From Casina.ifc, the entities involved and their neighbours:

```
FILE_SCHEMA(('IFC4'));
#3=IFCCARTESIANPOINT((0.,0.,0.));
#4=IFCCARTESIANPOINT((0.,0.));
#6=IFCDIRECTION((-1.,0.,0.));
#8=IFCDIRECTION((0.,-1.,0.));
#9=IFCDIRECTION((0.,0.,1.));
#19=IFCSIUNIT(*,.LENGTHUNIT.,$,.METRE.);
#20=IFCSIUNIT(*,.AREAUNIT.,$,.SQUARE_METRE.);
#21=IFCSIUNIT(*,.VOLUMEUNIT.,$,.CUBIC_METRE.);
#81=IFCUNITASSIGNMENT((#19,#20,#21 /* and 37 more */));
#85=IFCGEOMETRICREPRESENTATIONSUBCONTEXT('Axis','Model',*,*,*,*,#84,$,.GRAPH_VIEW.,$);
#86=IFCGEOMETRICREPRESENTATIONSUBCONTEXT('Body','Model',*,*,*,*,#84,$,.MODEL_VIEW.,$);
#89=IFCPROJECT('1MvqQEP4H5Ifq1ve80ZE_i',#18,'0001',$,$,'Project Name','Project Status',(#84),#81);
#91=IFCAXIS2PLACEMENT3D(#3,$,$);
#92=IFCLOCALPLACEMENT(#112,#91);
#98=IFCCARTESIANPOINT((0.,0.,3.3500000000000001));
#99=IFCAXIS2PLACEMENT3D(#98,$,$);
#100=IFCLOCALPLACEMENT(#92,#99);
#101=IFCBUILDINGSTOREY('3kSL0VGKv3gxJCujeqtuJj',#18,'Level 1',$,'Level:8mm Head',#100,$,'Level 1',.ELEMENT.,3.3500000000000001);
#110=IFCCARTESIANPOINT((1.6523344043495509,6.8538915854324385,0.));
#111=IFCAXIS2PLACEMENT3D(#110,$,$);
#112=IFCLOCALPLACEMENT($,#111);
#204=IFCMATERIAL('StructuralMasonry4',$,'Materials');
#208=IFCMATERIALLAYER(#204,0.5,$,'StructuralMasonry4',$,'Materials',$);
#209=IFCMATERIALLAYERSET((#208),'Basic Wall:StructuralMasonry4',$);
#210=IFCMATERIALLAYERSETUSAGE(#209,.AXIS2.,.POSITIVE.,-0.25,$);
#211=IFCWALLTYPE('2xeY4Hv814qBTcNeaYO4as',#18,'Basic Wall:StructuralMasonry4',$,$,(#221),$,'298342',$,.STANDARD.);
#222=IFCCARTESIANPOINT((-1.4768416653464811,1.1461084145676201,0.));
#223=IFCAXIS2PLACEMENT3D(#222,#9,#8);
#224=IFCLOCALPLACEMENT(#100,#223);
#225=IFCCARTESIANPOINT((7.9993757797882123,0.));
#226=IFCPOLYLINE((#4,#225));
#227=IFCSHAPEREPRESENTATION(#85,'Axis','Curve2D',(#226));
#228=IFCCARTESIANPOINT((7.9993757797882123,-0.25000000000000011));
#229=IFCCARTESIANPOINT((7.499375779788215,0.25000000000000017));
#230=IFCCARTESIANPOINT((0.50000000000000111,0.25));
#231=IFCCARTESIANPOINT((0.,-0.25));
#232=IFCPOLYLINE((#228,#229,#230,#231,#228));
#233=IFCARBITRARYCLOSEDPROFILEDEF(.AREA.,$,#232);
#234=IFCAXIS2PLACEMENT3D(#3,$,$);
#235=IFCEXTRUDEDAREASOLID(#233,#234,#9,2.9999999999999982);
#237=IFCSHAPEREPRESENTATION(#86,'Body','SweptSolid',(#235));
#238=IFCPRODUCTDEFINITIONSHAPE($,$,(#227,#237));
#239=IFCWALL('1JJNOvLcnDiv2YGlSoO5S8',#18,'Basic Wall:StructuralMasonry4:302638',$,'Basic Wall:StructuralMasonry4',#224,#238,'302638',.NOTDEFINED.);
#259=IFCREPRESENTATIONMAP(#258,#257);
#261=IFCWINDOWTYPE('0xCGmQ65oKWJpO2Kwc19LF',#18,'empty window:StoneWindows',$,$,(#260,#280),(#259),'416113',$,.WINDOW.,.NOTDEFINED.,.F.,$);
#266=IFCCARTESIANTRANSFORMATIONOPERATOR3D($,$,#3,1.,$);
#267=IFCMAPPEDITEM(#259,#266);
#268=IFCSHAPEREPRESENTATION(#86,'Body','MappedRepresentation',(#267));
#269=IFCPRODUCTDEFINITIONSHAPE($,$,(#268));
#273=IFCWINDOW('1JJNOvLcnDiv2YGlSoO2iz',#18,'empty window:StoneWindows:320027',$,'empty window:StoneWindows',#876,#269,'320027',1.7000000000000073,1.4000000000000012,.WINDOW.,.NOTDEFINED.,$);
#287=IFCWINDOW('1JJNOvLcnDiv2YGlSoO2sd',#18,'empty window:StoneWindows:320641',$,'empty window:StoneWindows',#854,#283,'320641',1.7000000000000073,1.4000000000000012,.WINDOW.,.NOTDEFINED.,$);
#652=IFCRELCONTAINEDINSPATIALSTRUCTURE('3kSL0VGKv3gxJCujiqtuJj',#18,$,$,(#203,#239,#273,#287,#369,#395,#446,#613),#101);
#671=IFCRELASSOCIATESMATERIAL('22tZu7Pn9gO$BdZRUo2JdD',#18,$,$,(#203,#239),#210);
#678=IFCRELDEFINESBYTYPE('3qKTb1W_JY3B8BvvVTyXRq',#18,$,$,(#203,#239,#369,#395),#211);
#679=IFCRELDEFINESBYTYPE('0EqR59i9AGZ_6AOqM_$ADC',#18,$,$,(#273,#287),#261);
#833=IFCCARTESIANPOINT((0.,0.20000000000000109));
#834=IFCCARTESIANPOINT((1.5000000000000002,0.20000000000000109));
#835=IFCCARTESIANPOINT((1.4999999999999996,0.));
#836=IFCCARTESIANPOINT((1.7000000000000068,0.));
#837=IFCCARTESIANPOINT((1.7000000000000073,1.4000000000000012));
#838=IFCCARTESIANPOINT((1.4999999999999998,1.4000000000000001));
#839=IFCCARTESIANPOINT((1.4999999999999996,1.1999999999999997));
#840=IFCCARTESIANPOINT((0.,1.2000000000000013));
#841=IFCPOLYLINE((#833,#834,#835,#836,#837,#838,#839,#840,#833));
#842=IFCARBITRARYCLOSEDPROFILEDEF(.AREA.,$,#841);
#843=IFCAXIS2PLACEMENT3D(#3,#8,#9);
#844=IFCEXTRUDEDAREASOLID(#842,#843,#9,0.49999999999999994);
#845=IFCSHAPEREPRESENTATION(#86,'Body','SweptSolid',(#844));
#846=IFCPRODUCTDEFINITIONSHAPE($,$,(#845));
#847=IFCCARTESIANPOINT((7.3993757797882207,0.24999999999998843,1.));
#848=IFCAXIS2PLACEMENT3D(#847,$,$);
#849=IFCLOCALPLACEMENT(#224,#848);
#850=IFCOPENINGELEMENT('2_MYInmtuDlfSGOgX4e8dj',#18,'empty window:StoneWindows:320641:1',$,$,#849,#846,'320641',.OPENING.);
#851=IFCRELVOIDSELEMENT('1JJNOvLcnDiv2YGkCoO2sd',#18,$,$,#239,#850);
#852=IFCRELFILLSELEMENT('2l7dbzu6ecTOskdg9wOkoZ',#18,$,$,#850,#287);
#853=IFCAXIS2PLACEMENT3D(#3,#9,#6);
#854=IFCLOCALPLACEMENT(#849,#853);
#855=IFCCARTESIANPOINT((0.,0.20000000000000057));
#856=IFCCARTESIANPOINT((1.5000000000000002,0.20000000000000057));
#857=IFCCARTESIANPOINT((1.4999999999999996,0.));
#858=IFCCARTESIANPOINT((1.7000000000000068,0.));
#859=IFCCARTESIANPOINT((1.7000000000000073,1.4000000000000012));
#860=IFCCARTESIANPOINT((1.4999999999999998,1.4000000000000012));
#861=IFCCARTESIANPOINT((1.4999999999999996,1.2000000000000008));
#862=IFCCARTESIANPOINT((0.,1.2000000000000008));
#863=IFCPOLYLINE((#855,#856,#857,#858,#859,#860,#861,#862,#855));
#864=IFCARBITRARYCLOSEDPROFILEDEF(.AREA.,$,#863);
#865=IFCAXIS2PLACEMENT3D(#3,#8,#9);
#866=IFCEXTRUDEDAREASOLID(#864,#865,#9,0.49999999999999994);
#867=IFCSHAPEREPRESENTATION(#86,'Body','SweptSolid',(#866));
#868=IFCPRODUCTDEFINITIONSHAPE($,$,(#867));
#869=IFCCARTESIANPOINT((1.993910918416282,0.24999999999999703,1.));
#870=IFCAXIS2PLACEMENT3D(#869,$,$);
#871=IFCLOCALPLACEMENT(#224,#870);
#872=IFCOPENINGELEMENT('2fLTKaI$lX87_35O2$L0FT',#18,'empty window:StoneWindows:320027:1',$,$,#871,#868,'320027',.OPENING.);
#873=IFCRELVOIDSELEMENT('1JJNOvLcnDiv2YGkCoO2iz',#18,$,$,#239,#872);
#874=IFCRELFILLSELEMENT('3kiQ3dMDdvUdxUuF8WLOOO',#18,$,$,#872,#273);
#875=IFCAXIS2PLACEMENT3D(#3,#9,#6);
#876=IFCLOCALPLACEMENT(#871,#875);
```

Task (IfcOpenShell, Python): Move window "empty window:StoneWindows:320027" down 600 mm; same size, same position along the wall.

```python
import numpy as np
import ifcopenshell
import ifcopenshell.api.geometry
import ifcopenshell.util.placement
import ifcopenshell.util.unit

model = ifcopenshell.open("Casina.ifc")
unit_scale = ifcopenshell.util.unit.calculate_unit_scale(model)

window = model.by_id(273)
opening = window.FillsVoids[0].RelatingOpeningElement
dz = -0.6

shift = np.array([0.0, 0.0, dz])
# The window is placed relative to its opening, so it follows when the opening moves.
matrix = ifcopenshell.util.placement.get_local_placement(opening.ObjectPlacement)
matrix[:3, 3] += shift
ifcopenshell.api.geometry.edit_object_placement(
    model, product=opening, matrix=matrix, is_si=False, should_transform_children=True
)

print(f"moved by {dz * unit_scale:+.3f} m")

model.write("Casina_v2.ifc")
```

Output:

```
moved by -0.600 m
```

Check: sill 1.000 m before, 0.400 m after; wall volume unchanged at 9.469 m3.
